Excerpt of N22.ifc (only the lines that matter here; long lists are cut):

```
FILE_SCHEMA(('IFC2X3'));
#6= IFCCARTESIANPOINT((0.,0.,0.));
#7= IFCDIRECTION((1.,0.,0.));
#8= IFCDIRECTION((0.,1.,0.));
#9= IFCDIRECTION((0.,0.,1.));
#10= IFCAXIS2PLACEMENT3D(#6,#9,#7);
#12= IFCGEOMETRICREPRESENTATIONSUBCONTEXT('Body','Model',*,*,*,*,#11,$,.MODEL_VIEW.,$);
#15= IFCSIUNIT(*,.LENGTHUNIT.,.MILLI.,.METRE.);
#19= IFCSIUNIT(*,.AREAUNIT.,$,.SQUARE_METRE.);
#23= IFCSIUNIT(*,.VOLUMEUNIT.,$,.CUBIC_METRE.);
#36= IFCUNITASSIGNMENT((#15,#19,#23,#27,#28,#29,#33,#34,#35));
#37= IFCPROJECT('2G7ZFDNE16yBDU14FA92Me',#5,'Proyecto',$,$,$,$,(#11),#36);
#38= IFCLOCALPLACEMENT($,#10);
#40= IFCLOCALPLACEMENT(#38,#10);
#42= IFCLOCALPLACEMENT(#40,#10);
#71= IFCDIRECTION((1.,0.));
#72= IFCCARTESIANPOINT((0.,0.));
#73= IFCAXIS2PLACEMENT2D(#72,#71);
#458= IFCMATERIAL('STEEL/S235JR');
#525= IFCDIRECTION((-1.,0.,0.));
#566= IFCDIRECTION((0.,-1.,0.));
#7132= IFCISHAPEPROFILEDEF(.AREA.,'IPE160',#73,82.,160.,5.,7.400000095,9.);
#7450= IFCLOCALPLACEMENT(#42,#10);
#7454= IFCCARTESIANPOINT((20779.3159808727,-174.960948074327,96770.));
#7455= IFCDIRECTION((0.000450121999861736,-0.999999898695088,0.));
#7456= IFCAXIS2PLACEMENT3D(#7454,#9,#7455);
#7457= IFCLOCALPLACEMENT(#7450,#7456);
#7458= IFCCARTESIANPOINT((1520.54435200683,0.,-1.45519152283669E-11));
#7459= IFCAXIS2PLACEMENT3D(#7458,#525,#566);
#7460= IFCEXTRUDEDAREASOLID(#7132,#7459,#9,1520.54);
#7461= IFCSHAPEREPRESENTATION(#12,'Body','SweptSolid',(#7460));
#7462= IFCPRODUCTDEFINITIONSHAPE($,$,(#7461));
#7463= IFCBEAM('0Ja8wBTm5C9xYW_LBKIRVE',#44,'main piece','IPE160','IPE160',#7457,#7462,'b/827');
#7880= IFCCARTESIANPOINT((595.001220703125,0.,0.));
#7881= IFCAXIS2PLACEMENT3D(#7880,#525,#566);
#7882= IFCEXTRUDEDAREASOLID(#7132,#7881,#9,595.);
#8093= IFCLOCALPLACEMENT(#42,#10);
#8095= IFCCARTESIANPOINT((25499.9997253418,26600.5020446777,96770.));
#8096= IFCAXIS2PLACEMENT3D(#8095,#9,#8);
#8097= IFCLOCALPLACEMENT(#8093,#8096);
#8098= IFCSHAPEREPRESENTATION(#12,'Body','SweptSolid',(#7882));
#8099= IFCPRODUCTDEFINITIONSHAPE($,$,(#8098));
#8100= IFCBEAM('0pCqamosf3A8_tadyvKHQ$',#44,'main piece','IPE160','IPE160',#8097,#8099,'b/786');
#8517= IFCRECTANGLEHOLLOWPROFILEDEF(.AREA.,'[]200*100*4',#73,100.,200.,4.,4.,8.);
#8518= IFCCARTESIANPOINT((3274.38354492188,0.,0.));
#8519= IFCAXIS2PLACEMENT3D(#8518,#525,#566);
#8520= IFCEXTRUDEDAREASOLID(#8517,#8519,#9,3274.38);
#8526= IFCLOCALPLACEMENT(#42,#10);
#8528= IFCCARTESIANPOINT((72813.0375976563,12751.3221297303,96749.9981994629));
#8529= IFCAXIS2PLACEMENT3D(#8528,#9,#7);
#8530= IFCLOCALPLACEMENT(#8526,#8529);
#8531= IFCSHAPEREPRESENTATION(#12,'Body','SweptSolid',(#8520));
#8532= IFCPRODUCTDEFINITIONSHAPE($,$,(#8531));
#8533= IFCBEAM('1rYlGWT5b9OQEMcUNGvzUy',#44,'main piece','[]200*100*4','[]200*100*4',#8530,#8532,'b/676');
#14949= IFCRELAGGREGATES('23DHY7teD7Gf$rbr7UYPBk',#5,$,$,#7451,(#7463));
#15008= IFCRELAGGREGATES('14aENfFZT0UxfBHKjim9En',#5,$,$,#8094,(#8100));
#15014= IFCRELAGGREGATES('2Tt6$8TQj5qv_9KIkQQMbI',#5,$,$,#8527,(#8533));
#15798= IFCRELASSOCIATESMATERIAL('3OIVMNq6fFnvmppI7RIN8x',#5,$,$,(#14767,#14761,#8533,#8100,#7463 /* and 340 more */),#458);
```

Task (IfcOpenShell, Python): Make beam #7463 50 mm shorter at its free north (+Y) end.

```python
import ifcopenshell
import ifcopenshell.util.representation

model = ifcopenshell.open("N22.ifc")

member = model.by_guid("0Ja8wBTm5C9xYW_LBKIRVE")
change = -50.0

# The extrusion runs towards the end named, so only its depth changes.
body = ifcopenshell.util.representation.get_representation(member, "Model", "Body")
solid = body.Items[0]
old_length = solid.Depth
solid.Depth += change

print(f"length {old_length:g} -> {solid.Depth:g}")

model.write("N22_rev.ifc")
```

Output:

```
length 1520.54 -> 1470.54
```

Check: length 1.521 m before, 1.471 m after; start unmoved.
